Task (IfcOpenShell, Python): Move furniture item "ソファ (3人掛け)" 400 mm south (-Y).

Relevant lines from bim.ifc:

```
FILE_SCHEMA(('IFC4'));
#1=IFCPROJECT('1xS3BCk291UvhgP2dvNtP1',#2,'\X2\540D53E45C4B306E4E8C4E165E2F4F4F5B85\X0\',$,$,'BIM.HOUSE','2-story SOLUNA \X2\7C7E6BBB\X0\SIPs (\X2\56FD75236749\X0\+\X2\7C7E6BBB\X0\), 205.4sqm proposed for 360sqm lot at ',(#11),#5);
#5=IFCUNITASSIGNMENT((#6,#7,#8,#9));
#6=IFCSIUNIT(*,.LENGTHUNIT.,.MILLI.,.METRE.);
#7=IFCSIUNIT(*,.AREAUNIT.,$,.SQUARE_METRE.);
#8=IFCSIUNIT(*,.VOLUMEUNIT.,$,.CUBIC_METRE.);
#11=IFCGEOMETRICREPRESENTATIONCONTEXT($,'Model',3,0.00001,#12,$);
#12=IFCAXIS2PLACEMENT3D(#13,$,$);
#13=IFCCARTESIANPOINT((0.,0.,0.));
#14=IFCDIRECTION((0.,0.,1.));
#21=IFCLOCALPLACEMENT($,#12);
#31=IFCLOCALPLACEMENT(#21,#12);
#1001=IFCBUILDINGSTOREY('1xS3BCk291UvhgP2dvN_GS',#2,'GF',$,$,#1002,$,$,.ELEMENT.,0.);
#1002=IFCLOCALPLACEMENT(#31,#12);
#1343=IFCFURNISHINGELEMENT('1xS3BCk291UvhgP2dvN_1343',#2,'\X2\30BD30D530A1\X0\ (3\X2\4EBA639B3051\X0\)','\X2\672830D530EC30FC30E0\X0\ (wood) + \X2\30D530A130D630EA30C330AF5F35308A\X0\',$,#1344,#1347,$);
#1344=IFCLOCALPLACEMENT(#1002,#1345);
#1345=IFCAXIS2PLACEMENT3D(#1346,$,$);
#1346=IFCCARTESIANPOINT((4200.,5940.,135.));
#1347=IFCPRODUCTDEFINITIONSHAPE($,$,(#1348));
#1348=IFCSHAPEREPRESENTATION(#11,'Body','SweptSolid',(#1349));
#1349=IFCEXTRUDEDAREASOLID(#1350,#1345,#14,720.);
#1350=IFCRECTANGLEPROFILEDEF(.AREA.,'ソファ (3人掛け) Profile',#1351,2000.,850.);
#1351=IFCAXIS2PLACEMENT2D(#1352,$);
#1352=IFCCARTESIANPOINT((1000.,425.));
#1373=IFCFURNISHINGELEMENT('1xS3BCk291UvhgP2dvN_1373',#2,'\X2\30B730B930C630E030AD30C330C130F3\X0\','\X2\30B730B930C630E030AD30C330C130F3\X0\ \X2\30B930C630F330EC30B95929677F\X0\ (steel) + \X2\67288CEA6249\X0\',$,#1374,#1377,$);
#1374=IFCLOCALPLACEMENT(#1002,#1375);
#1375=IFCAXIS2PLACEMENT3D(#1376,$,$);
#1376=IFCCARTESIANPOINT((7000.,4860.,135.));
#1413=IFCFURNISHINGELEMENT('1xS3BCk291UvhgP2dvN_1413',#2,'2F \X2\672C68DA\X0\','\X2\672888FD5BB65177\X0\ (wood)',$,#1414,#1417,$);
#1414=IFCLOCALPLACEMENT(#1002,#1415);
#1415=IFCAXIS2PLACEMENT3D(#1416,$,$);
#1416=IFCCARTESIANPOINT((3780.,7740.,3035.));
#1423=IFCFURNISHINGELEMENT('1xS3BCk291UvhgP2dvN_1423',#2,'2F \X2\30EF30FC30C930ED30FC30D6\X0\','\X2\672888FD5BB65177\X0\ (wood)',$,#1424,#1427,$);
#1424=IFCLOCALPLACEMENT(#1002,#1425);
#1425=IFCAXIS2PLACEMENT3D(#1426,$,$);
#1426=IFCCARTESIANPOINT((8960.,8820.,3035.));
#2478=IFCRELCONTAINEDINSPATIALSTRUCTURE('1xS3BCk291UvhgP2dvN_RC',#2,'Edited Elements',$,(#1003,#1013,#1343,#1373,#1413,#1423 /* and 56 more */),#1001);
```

```python
import ifcopenshell
import ifcopenshell.api.geometry
import ifcopenshell.util.placement

model = ifcopenshell.open("bim.ifc")

item = model.by_guid("1xS3BCk291UvhgP2dvN_1343")
matrix = ifcopenshell.util.placement.get_local_placement(item.ObjectPlacement)
matrix[1, 3] -= 400.0
ifcopenshell.api.geometry.edit_object_placement(model, product=item, matrix=matrix, is_si=False)

print(ifcopenshell.util.placement.get_local_placement(item.ObjectPlacement).round(3) + 0.0)

model.write("bim_edited.ifc")
```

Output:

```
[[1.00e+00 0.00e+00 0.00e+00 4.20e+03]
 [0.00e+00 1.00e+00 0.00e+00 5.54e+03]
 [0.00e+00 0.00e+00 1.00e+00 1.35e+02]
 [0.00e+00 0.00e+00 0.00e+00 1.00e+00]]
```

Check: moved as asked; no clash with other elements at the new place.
